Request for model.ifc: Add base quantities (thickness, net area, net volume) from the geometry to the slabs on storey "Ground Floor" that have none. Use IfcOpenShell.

First a look at what the model holds.

```python
import ifcopenshell
import ifcopenshell.util.element
import ifcopenshell.util.unit

model = ifcopenshell.open("model.ifc")
print(model.schema)
for unit_type in ("LENGTHUNIT", "AREAUNIT", "VOLUMEUNIT"):
    print(unit_type, ifcopenshell.util.unit.calculate_unit_scale(model, unit_type))
storey = next(s for s in model.by_type("IfcBuildingStorey") if s.Name == "Ground Floor")
slabs = [e for e in ifcopenshell.util.element.get_decomposition(storey) if e.is_a("IfcSlab")]
for e in sorted(slabs, key=lambda e: e.id()):
    print(e.id(), e.is_a(), e.Name, list(ifcopenshell.util.element.get_psets(e, qtos_only=True)), sep=" | ")
```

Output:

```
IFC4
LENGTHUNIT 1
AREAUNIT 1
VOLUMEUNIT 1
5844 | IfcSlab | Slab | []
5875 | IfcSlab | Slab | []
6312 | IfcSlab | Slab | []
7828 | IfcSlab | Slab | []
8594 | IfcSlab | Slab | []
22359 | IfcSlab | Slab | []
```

```python
import ifcopenshell
import ifcopenshell.api.pset
import ifcopenshell.geom
import ifcopenshell.util.element
import ifcopenshell.util.shape
import ifcopenshell.util.unit

model = ifcopenshell.open("model.ifc")
unit_scale = ifcopenshell.util.unit.calculate_unit_scale(model)
area_scale = ifcopenshell.util.unit.calculate_unit_scale(model, "AREAUNIT")
volume_scale = ifcopenshell.util.unit.calculate_unit_scale(model, "VOLUMEUNIT")
settings = ifcopenshell.geom.settings()

storey = next(s for s in model.by_type("IfcBuildingStorey") if s.Name == "Ground Floor")
slabs = [e for e in ifcopenshell.util.element.get_decomposition(storey) if e.is_a("IfcSlab")]

for e in sorted(slabs, key=lambda e: e.id()):
    if ifcopenshell.util.element.get_psets(e, qtos_only=True, should_inherit=False):
        continue
    # Geometry comes back in metres, in the element's own axes.
    shape = ifcopenshell.geom.create_shape(settings, e)
    values = {
        "Width": ifcopenshell.util.shape.get_z(shape.geometry) / unit_scale,
        "NetArea": ifcopenshell.util.shape.get_footprint_area(shape.geometry) / area_scale,
        "NetVolume": ifcopenshell.util.shape.get_volume(shape.geometry) / volume_scale,
    }
    qto = ifcopenshell.api.pset.add_qto(model, product=e, name="Qto_SlabBaseQuantities")
    ifcopenshell.api.pset.edit_qto(model, qto=qto, properties=values)
    print(e.id(), {k: round(v, 3) for k, v in values.items()})

model.write("model_v2.ifc")
```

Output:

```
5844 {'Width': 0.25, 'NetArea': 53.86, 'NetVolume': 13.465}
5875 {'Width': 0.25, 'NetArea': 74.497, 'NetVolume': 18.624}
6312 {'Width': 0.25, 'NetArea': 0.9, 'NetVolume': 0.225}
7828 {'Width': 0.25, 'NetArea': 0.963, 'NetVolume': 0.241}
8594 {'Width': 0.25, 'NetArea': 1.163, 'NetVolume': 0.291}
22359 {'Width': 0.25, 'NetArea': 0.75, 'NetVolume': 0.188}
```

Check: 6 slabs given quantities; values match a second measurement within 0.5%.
